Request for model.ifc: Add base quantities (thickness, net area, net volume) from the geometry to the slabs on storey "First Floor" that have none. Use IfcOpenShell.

First a look at what the model holds.

```python
import ifcopenshell
import ifcopenshell.util.element
import ifcopenshell.util.unit

model = ifcopenshell.open("model.ifc")
print(model.schema)
for unit_type in ("LENGTHUNIT", "AREAUNIT", "VOLUMEUNIT"):
    print(unit_type, ifcopenshell.util.unit.calculate_unit_scale(model, unit_type))
storey = next(s for s in model.by_type("IfcBuildingStorey") if s.Name == "First Floor")
slabs = [e for e in ifcopenshell.util.element.get_decomposition(storey) if e.is_a("IfcSlab")]
for e in sorted(slabs, key=lambda e: e.id()):
    print(e.id(), e.is_a(), e.Name, list(ifcopenshell.util.element.get_psets(e, qtos_only=True)), sep=" | ")
```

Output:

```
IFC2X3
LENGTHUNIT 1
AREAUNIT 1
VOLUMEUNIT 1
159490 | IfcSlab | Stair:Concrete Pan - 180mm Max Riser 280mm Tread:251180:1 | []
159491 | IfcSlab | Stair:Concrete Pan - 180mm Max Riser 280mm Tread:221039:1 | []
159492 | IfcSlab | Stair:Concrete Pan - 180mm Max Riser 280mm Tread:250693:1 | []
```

```python
import ifcopenshell
import ifcopenshell.api.pset
import ifcopenshell.geom
import ifcopenshell.util.element
import ifcopenshell.util.shape
import ifcopenshell.util.unit

model = ifcopenshell.open("model.ifc")
unit_scale = ifcopenshell.util.unit.calculate_unit_scale(model)
area_scale = ifcopenshell.util.unit.calculate_unit_scale(model, "AREAUNIT")
volume_scale = ifcopenshell.util.unit.calculate_unit_scale(model, "VOLUMEUNIT")
settings = ifcopenshell.geom.settings()

storey = next(s for s in model.by_type("IfcBuildingStorey") if s.Name == "First Floor")
slabs = [e for e in ifcopenshell.util.element.get_decomposition(storey) if e.is_a("IfcSlab")]

for e in sorted(slabs, key=lambda e: e.id()):
    if ifcopenshell.util.element.get_psets(e, qtos_only=True, should_inherit=False):
        continue
    # Geometry comes back in metres, in the element's own axes.
    shape = ifcopenshell.geom.create_shape(settings, e)
    values = {
        "Width": ifcopenshell.util.shape.get_z(shape.geometry) / unit_scale,
        "NetArea": ifcopenshell.util.shape.get_footprint_area(shape.geometry) / area_scale,
        "NetVolume": ifcopenshell.util.shape.get_volume(shape.geometry) / volume_scale,
    }
    qto = ifcopenshell.api.pset.add_qto(model, product=e, name="BaseQuantities")
    ifcopenshell.api.pset.edit_qto(model, qto=qto, properties=values)
    print(e.id(), {k: round(v, 3) for k, v in values.items()})

model.write("model_edited.ifc")
```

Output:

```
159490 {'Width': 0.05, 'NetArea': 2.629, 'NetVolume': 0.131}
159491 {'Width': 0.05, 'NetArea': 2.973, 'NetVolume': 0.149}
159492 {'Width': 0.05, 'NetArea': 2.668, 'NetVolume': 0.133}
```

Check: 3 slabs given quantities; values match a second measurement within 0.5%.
